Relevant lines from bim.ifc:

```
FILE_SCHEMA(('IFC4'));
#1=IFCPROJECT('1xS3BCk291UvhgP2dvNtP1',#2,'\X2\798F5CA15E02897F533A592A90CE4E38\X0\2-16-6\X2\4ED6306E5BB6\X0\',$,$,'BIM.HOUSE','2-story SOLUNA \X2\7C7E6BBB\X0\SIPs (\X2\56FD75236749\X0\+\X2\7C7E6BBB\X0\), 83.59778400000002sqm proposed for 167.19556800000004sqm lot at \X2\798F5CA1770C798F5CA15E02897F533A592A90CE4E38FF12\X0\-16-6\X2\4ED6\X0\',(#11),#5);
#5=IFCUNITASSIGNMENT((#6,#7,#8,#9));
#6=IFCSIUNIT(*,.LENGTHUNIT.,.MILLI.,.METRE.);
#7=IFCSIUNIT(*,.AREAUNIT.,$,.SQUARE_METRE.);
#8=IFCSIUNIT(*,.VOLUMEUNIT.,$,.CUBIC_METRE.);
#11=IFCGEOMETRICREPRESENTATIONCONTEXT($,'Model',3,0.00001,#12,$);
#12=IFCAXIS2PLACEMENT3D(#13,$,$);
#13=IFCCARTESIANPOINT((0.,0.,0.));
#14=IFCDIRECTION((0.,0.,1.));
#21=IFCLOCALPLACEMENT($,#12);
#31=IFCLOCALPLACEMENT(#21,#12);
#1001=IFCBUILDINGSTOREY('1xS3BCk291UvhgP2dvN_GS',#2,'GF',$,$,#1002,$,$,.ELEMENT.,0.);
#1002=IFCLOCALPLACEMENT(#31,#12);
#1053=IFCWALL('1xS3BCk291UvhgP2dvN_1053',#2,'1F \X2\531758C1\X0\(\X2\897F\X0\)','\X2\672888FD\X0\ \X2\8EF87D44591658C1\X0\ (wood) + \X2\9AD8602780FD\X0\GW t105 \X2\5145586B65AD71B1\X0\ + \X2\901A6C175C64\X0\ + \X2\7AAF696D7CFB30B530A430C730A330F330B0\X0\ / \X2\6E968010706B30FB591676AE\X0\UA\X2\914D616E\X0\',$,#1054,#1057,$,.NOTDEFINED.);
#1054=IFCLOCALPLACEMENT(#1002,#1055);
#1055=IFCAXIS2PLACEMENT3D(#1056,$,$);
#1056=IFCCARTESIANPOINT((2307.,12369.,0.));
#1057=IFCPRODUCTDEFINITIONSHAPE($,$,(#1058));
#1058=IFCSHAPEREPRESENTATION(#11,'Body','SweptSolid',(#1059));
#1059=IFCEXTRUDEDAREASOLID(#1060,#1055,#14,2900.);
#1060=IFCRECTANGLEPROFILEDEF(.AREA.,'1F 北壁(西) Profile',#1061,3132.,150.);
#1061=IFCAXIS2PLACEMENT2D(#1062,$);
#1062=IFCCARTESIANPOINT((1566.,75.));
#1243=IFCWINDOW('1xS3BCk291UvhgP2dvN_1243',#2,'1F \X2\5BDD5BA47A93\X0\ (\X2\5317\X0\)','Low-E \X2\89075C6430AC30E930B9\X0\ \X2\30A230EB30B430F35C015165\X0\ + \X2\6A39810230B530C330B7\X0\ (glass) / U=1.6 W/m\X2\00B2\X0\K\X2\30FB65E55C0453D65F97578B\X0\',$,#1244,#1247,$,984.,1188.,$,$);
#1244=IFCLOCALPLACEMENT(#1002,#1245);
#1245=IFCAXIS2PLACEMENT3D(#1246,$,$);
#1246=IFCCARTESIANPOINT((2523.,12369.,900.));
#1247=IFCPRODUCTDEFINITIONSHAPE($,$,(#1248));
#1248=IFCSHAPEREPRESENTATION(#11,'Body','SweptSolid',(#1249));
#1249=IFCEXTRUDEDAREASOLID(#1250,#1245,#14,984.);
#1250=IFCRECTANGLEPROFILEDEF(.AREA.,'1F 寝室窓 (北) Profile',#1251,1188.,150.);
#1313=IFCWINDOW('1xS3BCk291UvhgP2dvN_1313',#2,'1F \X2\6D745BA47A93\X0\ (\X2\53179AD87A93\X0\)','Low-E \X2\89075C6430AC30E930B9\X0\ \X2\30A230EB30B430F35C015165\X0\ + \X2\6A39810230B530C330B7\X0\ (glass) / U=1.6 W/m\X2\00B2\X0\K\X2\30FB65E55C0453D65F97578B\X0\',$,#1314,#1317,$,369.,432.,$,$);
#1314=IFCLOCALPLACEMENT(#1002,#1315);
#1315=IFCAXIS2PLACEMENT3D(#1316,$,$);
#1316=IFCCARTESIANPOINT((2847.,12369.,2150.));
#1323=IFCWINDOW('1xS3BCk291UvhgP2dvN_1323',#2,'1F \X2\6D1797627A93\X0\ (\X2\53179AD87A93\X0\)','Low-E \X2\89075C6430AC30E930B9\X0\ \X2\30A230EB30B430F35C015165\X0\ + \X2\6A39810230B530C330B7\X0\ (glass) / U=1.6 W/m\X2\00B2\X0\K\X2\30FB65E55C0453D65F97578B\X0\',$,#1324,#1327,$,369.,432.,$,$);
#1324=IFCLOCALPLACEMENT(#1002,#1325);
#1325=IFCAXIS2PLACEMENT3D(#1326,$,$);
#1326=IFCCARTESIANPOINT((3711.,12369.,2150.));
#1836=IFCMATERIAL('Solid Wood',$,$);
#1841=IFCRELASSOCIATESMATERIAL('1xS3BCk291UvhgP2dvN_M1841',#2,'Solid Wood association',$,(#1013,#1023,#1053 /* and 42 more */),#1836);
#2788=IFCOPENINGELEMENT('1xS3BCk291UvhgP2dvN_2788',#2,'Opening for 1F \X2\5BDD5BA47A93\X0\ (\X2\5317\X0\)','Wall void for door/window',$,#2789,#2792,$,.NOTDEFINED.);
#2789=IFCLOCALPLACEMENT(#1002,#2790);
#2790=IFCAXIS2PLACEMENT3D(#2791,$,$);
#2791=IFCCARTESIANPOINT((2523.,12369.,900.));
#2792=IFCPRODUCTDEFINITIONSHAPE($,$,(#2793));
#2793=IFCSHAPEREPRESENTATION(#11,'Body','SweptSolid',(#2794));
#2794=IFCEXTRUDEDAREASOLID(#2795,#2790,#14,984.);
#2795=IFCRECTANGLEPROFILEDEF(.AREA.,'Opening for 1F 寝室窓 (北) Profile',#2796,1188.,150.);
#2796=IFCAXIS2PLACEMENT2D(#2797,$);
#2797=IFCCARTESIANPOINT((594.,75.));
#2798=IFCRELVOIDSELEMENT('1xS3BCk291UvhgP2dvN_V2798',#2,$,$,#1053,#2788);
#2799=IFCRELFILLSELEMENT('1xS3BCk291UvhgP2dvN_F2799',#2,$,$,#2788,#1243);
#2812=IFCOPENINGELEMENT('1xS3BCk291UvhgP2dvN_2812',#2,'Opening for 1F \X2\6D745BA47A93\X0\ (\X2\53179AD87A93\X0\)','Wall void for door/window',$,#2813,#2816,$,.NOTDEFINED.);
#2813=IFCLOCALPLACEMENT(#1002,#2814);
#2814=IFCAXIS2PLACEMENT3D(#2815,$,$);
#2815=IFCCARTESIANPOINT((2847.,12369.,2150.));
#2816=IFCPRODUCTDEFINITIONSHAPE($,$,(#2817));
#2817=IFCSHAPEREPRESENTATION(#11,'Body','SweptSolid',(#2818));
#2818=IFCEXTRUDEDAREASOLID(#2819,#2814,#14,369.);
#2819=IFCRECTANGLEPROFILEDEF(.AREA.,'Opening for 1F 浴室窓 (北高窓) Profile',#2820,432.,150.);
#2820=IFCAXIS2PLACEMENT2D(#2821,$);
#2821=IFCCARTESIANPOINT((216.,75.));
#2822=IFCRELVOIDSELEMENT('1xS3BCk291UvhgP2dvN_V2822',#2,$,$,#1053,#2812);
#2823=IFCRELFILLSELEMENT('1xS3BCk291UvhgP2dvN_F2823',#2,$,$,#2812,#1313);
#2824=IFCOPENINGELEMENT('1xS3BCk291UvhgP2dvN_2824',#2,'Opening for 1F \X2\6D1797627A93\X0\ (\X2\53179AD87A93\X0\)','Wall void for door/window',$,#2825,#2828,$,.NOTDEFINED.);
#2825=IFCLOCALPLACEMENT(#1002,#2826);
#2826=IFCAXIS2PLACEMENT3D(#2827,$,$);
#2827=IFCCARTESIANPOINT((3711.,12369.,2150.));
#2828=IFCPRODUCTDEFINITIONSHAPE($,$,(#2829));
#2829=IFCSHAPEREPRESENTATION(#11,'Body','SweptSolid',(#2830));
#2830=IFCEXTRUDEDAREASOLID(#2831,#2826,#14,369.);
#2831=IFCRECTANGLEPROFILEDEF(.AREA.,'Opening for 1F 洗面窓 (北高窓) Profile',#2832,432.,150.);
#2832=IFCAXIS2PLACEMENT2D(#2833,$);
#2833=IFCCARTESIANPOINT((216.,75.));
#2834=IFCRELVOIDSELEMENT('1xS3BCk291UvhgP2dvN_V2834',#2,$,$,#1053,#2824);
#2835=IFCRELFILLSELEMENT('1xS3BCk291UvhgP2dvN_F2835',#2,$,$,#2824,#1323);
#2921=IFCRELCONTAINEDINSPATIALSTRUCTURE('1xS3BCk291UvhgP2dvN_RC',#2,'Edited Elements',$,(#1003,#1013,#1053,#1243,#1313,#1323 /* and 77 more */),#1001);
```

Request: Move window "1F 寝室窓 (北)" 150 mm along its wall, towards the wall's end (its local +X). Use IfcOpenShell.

```python
import ifcopenshell
import ifcopenshell.api.geometry
import ifcopenshell.util.placement

model = ifcopenshell.open("bim.ifc")

window = model.by_guid("1xS3BCk291UvhgP2dvN_1243")
opening = window.FillsVoids[0].RelatingOpeningElement
wall = opening.VoidsElements[0].RelatingBuildingElement

wall_matrix = ifcopenshell.util.placement.get_local_placement(wall.ObjectPlacement)
shift = wall_matrix[:3, 0] * 150.0
before = ifcopenshell.util.placement.get_local_placement(window.ObjectPlacement)[:3, 3].copy()

# The window is not placed relative to its opening, so move both.
for product in (opening, window):
    matrix = ifcopenshell.util.placement.get_local_placement(product.ObjectPlacement)
    matrix[:3, 3] += shift
    ifcopenshell.api.geometry.edit_object_placement(model, product=product, matrix=matrix, is_si=False)

after = ifcopenshell.util.placement.get_local_placement(window.ObjectPlacement)[:3, 3]
print("window moved by", (after - before).round(3) + 0.0)

model.write("bim_updated.ifc")
```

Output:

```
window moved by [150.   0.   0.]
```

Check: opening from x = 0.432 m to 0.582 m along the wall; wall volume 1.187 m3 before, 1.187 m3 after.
